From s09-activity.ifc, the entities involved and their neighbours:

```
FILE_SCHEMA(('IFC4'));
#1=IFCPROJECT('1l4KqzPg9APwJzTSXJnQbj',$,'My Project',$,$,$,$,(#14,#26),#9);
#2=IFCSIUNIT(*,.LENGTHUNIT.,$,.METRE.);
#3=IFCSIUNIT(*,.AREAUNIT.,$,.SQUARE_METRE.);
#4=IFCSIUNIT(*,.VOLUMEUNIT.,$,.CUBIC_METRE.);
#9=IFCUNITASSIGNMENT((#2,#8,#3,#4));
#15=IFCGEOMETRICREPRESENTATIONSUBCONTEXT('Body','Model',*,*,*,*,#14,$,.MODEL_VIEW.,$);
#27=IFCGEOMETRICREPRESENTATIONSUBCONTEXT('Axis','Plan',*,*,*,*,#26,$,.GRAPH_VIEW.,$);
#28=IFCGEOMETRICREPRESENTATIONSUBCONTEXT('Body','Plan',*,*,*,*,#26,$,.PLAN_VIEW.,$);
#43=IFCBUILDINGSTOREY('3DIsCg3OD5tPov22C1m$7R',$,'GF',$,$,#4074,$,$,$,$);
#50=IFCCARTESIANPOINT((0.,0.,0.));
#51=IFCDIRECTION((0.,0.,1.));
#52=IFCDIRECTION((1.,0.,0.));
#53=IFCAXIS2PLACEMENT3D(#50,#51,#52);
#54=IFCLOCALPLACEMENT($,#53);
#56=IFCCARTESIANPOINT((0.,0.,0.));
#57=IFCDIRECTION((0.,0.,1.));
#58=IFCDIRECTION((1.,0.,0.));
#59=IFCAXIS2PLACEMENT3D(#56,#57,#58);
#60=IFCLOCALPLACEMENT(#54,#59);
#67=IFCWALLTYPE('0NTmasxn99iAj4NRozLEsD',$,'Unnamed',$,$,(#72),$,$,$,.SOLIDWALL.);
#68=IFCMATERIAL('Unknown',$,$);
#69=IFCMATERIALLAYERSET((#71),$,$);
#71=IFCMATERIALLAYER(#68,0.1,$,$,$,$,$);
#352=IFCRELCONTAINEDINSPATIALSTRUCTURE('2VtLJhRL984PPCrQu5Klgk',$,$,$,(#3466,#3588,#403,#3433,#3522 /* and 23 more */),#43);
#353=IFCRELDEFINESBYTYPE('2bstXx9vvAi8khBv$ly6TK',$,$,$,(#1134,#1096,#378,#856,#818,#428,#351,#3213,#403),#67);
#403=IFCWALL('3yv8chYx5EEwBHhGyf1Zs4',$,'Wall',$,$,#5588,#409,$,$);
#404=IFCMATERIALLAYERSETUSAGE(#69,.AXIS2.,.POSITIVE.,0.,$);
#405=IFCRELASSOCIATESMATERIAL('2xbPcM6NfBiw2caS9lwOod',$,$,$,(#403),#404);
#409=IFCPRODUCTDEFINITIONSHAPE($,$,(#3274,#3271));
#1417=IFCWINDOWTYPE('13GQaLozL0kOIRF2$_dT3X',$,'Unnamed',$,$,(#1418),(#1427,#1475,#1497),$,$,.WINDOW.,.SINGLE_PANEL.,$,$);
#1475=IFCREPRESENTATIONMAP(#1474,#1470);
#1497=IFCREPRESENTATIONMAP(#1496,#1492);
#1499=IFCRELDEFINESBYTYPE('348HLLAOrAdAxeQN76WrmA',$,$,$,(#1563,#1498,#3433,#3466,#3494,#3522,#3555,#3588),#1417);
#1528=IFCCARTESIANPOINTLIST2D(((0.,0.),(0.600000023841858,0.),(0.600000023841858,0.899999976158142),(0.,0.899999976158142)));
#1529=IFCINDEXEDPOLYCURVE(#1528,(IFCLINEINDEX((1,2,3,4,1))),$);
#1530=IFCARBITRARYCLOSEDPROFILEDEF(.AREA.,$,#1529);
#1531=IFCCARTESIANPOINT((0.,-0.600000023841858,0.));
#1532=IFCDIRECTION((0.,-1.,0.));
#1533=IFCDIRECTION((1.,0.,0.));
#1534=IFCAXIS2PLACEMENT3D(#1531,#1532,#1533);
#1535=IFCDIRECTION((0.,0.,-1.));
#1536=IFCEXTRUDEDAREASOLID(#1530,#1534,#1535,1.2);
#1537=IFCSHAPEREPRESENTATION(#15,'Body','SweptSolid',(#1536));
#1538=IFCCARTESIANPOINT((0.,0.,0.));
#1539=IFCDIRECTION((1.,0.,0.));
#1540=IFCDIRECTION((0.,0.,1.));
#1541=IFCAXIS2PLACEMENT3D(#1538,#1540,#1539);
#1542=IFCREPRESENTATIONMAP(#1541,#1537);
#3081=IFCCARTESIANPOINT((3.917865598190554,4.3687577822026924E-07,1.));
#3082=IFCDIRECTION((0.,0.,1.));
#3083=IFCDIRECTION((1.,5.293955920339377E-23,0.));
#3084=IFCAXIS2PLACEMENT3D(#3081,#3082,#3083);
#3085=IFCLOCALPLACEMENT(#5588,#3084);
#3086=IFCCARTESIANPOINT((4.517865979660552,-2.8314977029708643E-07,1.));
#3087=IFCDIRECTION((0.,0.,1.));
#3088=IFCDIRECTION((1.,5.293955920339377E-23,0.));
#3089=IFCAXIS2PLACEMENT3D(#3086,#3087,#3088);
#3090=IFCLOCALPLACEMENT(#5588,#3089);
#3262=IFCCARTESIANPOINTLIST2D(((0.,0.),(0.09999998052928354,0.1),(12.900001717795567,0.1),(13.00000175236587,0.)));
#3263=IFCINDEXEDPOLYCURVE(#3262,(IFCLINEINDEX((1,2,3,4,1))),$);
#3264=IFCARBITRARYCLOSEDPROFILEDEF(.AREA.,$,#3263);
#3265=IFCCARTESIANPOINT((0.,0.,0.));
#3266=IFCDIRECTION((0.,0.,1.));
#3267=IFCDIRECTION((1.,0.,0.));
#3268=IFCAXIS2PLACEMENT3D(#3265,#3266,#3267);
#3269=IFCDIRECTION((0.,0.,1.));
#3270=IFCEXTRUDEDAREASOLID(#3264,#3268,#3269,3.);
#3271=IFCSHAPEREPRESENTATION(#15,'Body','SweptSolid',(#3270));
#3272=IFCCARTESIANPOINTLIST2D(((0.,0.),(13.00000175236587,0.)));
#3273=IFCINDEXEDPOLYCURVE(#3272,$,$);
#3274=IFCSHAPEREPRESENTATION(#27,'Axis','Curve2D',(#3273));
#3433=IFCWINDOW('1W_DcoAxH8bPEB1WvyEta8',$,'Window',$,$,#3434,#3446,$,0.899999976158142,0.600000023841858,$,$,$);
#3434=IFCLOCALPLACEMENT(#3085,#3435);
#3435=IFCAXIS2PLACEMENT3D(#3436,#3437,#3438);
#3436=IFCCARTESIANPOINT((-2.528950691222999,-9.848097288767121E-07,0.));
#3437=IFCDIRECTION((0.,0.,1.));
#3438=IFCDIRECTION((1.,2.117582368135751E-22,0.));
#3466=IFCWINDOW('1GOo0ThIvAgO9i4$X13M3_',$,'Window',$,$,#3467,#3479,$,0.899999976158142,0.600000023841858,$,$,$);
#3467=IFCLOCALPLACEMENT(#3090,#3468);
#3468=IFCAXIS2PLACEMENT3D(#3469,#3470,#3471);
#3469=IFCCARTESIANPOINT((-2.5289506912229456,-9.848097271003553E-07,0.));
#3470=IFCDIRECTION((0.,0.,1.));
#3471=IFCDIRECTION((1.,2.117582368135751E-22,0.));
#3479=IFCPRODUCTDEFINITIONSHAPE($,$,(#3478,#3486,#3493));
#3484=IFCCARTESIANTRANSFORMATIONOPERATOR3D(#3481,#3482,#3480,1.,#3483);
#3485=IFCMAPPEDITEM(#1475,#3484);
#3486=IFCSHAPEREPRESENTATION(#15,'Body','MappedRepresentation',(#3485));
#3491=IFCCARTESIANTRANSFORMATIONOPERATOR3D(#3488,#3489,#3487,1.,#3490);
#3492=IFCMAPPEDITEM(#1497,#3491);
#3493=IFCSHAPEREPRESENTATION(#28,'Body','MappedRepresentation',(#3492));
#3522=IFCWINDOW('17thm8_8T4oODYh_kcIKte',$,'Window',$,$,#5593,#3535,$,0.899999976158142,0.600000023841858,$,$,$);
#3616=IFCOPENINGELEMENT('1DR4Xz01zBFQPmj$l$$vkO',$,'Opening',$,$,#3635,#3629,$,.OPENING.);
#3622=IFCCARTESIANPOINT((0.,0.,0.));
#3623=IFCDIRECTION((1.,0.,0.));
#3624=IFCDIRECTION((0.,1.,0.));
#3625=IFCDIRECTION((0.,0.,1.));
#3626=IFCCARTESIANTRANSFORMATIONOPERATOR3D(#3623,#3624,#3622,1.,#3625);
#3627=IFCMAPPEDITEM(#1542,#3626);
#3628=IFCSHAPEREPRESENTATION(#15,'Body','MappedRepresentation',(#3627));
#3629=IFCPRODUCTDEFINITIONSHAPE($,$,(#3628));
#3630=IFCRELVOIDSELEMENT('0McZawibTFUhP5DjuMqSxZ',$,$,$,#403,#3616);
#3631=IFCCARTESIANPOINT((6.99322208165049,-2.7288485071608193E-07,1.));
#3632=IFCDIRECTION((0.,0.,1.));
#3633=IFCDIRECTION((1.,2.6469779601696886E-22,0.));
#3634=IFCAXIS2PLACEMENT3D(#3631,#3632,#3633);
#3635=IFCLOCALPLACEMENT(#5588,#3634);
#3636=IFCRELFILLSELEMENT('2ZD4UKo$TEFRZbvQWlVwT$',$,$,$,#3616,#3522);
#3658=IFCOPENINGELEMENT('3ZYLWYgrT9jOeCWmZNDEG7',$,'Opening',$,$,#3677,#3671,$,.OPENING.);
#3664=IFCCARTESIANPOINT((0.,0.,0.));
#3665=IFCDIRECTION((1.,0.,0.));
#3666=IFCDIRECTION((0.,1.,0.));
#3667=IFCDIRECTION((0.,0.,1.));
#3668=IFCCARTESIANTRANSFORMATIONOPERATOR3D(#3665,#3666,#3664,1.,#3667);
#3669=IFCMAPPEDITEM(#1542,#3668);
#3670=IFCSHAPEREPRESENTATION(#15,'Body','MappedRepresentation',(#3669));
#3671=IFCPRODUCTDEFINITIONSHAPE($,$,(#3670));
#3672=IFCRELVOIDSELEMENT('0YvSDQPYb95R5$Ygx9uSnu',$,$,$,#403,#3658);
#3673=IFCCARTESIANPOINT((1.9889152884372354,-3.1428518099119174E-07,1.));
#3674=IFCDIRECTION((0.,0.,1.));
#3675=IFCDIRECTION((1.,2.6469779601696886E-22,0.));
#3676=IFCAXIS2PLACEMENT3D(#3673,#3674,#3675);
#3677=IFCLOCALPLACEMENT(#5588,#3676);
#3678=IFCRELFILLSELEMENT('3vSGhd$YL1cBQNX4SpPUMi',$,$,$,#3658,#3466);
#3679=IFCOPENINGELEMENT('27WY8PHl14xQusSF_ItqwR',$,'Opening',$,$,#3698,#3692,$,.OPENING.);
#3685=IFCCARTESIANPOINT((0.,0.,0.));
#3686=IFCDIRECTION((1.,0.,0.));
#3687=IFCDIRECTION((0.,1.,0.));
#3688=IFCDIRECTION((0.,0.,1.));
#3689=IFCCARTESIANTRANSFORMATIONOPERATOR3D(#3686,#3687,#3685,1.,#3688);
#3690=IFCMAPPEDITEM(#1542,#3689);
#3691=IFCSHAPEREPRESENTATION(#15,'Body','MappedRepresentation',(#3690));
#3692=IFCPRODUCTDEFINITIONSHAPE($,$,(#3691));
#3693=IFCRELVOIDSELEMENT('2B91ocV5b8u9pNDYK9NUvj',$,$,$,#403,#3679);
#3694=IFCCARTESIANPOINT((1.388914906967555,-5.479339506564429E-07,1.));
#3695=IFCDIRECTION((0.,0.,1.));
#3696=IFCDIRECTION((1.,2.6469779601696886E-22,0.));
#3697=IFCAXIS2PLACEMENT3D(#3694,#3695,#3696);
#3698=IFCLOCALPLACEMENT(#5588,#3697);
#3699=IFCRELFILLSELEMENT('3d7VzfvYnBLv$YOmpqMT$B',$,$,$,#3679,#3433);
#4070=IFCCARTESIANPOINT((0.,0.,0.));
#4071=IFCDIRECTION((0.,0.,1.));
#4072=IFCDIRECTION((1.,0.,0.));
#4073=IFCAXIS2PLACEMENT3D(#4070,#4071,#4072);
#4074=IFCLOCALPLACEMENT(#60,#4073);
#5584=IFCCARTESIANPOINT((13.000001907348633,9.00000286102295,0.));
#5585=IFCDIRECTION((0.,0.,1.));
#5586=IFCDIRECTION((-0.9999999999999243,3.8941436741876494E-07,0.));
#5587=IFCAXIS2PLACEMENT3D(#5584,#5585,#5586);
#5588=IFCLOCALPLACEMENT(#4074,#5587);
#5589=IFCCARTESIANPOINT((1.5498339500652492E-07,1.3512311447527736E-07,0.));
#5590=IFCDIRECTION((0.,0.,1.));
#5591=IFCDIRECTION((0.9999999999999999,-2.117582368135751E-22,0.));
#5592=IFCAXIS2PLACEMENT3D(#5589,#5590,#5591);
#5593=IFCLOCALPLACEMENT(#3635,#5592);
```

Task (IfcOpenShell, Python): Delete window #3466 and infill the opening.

```python
import ifcopenshell
import ifcopenshell.api.feature
import ifcopenshell.api.root
import ifcopenshell.geom
import ifcopenshell.util.shape

model = ifcopenshell.open("s09-activity.ifc")
settings = ifcopenshell.geom.settings()


def volume(element):
    """Net volume in cubic metres, openings subtracted."""
    shape = ifcopenshell.geom.create_shape(settings, element)
    return ifcopenshell.util.shape.get_volume(shape.geometry)


window = model.by_id(3466)
opening = window.FillsVoids[0].RelatingOpeningElement
wall = opening.VoidsElements[0].RelatingBuildingElement
before = volume(wall)

ifcopenshell.api.root.remove_product(model, product=window)
ifcopenshell.api.feature.remove_feature(model, feature=opening)

after = volume(wall)

print(f"wall volume {before:.3f} -> {after:.3f} m3")

model.write("s09-activity-out.ifc")
```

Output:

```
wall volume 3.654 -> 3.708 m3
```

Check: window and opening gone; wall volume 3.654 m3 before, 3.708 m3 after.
